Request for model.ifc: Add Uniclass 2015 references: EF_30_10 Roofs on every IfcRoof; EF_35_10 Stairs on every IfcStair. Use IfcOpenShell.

First a look at what the model holds.

```python
import ifcopenshell

model = ifcopenshell.open("model.ifc")
print(model.schema)
print("classifications:", [c.Name for c in model.by_type("IfcClassification")])
for ifc_class in ("IfcDoor", "IfcRoof", "IfcStair", "IfcWall", "IfcWindow"):
    print(ifc_class, len(model.by_type(ifc_class)))
```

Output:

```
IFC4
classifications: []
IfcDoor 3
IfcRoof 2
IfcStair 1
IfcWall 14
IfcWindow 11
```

```python
import ifcopenshell
import ifcopenshell.api.classification

model = ifcopenshell.open("model.ifc")

system = ifcopenshell.api.classification.add_classification(model, classification="Uniclass 2015")

codes = {
    "IfcRoof": ("EF_30_10", "Roofs"),
    "IfcStair": ("EF_35_10", "Stairs"),
}
for ifc_class, (code, name) in codes.items():
    products = model.by_type(ifc_class)
    ifcopenshell.api.classification.add_reference(
        model, products=products, classification=system, identification=code, name=name
    )
    print(code, len(products))

model.write("model_rev.ifc")
```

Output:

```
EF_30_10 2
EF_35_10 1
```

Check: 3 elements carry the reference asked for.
